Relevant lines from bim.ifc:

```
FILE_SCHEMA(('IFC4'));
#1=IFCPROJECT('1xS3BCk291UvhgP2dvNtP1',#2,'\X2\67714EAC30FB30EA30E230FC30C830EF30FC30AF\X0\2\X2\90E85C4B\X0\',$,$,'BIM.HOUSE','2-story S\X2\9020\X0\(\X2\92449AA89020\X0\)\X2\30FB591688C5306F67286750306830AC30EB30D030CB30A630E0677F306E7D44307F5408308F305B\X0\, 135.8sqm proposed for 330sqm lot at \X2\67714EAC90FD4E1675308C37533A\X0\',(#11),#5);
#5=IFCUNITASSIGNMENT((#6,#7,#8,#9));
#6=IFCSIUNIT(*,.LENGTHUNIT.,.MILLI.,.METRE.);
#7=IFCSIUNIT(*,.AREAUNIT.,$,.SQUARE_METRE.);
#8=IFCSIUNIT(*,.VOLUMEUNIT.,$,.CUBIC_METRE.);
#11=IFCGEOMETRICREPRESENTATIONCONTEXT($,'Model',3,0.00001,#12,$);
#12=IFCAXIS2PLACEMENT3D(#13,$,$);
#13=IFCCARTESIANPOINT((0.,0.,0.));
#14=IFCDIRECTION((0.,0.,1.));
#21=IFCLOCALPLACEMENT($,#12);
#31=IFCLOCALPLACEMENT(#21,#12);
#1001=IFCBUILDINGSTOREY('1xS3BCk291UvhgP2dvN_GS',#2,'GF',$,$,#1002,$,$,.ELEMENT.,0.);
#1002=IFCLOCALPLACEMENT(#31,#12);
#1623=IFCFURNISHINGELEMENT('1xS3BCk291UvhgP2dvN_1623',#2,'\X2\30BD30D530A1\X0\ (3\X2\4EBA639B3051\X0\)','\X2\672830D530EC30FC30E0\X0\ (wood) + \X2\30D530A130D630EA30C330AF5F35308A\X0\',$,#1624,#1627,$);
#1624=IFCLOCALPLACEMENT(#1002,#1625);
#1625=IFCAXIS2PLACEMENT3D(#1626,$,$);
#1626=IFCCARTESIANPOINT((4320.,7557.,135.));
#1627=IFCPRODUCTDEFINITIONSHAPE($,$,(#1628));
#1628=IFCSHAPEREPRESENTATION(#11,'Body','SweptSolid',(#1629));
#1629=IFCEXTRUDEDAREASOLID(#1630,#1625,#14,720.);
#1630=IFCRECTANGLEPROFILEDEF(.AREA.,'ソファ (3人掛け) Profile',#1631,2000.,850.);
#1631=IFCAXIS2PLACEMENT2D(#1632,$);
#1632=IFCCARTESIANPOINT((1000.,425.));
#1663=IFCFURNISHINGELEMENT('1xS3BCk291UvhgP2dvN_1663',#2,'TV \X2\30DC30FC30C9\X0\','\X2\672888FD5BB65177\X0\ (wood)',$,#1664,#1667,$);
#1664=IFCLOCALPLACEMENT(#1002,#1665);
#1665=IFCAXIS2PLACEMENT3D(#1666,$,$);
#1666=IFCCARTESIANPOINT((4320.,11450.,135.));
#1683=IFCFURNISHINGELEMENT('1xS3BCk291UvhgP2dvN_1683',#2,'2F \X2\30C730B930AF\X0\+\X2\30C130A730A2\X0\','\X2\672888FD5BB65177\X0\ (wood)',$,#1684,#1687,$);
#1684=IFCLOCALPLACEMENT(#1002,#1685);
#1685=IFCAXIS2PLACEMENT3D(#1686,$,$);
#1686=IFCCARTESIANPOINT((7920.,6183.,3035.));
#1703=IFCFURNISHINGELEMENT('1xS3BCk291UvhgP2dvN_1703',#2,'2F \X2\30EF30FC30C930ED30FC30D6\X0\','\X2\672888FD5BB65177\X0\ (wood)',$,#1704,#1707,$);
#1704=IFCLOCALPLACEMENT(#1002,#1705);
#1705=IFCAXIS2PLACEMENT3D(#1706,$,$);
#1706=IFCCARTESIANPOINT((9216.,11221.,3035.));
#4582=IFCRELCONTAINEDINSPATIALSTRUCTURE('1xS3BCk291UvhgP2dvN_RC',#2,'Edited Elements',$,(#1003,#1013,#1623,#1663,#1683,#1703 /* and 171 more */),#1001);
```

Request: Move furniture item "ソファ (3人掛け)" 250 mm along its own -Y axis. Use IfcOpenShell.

```python
import ifcopenshell
import ifcopenshell.api.geometry
import ifcopenshell.util.placement
import ifcopenshell.util.unit

model = ifcopenshell.open("bim.ifc")
unit_scale = ifcopenshell.util.unit.calculate_unit_scale(model)

item = model.by_guid("1xS3BCk291UvhgP2dvN_1623")
matrix = ifcopenshell.util.placement.get_local_placement(item.ObjectPlacement)
matrix[:3, 3] -= matrix[:3, 1] * 0.25 / unit_scale
ifcopenshell.api.geometry.edit_object_placement(model, product=item, matrix=matrix, is_si=False)

print(ifcopenshell.util.placement.get_local_placement(item.ObjectPlacement).round(3) + 0.0)

model.write("bim_rev.ifc")
```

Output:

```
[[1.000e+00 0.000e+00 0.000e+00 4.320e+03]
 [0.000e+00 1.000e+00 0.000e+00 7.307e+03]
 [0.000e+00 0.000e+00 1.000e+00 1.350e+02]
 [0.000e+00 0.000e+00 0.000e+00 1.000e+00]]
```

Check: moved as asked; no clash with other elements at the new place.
